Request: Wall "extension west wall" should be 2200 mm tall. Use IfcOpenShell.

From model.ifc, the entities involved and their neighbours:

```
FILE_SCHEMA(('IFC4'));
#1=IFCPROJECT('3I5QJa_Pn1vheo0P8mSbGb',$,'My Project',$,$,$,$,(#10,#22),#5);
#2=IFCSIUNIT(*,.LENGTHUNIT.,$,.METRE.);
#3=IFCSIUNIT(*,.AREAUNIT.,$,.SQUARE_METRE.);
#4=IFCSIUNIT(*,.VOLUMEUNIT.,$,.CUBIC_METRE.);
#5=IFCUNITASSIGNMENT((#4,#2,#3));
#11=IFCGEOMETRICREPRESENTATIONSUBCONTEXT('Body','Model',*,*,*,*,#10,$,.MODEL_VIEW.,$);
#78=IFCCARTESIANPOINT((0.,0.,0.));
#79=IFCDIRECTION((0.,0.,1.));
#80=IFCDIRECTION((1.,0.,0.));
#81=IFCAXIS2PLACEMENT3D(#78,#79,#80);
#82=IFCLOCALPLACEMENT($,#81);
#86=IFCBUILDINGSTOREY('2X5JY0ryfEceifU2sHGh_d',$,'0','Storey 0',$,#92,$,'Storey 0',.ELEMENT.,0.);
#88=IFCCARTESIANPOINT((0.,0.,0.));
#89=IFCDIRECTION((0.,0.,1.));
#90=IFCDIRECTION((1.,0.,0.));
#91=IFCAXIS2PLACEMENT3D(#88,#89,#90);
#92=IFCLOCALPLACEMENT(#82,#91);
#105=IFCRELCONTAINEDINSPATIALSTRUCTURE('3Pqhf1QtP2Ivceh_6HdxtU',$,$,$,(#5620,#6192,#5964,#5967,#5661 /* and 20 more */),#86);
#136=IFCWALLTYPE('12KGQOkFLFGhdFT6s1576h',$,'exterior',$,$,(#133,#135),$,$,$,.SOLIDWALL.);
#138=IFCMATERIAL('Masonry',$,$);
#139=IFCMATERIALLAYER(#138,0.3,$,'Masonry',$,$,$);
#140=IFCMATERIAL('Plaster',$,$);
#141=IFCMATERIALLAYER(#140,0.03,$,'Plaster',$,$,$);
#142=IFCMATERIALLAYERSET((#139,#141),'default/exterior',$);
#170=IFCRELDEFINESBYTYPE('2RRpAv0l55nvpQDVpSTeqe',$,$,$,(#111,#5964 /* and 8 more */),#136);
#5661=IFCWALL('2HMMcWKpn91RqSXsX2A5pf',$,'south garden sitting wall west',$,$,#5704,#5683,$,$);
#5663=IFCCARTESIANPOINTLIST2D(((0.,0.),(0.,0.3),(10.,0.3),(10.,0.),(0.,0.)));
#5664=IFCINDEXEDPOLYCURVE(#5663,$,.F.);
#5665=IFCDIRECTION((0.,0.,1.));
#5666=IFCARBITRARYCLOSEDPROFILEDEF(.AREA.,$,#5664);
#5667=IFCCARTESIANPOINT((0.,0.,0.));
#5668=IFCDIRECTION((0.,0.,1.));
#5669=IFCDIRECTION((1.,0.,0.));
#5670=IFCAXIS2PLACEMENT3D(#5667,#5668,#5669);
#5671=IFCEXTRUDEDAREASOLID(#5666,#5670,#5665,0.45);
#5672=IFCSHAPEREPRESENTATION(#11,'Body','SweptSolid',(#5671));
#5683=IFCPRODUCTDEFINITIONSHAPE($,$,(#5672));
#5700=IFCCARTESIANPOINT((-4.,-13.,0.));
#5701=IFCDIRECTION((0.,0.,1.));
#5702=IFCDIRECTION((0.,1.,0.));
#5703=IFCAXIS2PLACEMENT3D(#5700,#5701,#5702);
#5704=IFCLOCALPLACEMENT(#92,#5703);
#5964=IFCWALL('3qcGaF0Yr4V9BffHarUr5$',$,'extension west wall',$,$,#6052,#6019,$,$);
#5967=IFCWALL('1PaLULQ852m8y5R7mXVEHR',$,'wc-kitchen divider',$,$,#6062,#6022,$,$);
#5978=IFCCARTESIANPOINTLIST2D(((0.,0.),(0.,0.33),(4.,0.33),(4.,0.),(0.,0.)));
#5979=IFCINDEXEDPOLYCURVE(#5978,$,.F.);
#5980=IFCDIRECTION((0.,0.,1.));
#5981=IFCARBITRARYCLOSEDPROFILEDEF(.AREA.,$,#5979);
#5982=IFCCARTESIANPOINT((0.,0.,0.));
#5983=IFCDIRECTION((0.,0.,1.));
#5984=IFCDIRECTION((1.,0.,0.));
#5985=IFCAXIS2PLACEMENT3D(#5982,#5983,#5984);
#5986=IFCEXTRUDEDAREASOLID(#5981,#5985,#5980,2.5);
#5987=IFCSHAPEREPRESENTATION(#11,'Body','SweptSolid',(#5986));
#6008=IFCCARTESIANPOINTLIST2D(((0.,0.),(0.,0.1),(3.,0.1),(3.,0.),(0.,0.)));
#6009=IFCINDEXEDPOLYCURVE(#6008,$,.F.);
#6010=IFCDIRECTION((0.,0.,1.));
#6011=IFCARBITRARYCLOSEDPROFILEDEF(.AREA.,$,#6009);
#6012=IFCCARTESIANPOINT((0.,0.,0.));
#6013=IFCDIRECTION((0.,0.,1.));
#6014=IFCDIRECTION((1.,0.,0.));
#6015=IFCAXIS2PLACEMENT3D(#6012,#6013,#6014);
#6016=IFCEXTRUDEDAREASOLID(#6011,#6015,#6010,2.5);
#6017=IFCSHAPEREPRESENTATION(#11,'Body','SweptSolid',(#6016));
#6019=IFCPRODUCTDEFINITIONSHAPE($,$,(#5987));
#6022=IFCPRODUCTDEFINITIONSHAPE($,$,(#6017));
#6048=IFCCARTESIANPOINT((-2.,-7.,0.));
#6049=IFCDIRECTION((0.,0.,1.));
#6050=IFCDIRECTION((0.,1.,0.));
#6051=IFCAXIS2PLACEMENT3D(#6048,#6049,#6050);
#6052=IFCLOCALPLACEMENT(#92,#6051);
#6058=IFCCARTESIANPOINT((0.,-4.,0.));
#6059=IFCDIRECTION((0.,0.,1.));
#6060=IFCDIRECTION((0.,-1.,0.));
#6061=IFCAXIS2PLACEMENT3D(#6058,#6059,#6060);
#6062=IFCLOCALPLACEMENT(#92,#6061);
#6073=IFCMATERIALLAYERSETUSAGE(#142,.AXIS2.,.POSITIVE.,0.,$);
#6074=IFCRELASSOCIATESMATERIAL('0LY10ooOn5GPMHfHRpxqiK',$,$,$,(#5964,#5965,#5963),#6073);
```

```python
import ifcopenshell
import ifcopenshell.geom
import ifcopenshell.util.representation
import ifcopenshell.util.shape
import ifcopenshell.util.unit

model = ifcopenshell.open("model.ifc")
unit_scale = ifcopenshell.util.unit.calculate_unit_scale(model)
settings = ifcopenshell.geom.settings()


def volume(element):
    """Net volume in cubic metres, openings subtracted."""
    shape = ifcopenshell.geom.create_shape(settings, element)
    return ifcopenshell.util.shape.get_volume(shape.geometry)


wall = model.by_guid("3qcGaF0Yr4V9BffHarUr5$")
before = volume(wall)

body = ifcopenshell.util.representation.get_representation(wall, "Model", "Body")
solid = body.Items[0]
old_height = solid.Depth
solid.Depth = 2.2 / unit_scale
after = volume(wall)

print(f"height {old_height:g} -> {solid.Depth:g}, volume {before:.3f} -> {after:.3f} m3")

model.write("model_rev.ifc")
```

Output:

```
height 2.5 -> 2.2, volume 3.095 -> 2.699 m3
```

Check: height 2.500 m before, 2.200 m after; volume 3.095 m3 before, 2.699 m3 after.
